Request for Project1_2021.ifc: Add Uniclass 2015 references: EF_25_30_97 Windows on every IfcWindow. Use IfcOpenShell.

First a look at what the model holds.

```python
import ifcopenshell

model = ifcopenshell.open("Project1_2021.ifc")
print(model.schema)
print("classifications:", [c.Name for c in model.by_type("IfcClassification")])
for ifc_class in ("IfcDoor", "IfcRoof", "IfcStair", "IfcWall", "IfcWindow"):
    print(ifc_class, len(model.by_type(ifc_class)))
```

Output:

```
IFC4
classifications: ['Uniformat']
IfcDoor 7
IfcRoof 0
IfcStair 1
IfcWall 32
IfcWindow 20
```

```python
import ifcopenshell
import ifcopenshell.api.classification

model = ifcopenshell.open("Project1_2021.ifc")

system = ifcopenshell.api.classification.add_classification(model, classification="Uniclass 2015")

codes = {
    "IfcWindow": ("EF_25_30_97", "Windows"),
}
for ifc_class, (code, name) in codes.items():
    products = model.by_type(ifc_class)
    ifcopenshell.api.classification.add_reference(
        model, products=products, classification=system, identification=code, name=name
    )
    print(code, len(products))

model.write("Project1_2021_updated.ifc")
```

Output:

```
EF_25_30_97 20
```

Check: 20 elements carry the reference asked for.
